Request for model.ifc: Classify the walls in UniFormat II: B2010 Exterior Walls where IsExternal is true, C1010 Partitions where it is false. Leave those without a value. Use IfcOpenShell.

First a look at what the model holds.

```python
import ifcopenshell
import ifcopenshell.util.element

model = ifcopenshell.open("model.ifc")
print(model.schema)
print("classifications:", [c.Name for c in model.by_type("IfcClassification")])
values = [ifcopenshell.util.element.get_pset(e, "Pset_WallCommon", "IsExternal") for e in model.by_type("IfcWall")]
for value in (True, False, None):
    print("IsExternal", value, values.count(value))
```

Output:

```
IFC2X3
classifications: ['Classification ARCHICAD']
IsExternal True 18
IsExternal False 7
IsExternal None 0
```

```python
import ifcopenshell
import ifcopenshell.api.classification
import ifcopenshell.util.element

model = ifcopenshell.open("model.ifc")

# IFC2X3 requires Source and Edition and has no link from the project to the system.
system = model.create_entity("IfcClassification", Source="ASTM", Edition="E1557", Name="UniFormat II")

walls = model.by_type("IfcWall")
external = {e: ifcopenshell.util.element.get_pset(e, "Pset_WallCommon", "IsExternal") for e in walls}
for flag, code, name in ((True, "B2010", "Exterior Walls"), (False, "C1010", "Partitions")):
    products = [e for e in walls if external[e] is flag]
    ifcopenshell.api.classification.add_reference(
        model, products=products, classification=system, identification=code, name=name
    )
    print(code, len(products))

model.write("model_edited.ifc")
```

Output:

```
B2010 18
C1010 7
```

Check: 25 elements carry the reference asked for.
